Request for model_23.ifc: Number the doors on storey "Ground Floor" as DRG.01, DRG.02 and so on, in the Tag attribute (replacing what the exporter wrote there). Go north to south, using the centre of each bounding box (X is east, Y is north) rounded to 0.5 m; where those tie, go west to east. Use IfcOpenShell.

First a look at what the model holds.

```python
import ifcopenshell
import ifcopenshell.util.element
import ifcopenshell.util.placement

model = ifcopenshell.open("model_23.ifc")
print(model.schema)
storey = next(s for s in model.by_type("IfcBuildingStorey") if s.Name == "Ground Floor")
doors = [e for e in ifcopenshell.util.element.get_decomposition(storey) if e.is_a("IfcDoor")]
for e in sorted(doors, key=lambda e: e.id()):
    origin = ifcopenshell.util.placement.get_local_placement(e.ObjectPlacement)[:3, 3]
    print(e.id(), e.Tag, e.Name, origin.round(2) + 0.0, sep=" | ")
```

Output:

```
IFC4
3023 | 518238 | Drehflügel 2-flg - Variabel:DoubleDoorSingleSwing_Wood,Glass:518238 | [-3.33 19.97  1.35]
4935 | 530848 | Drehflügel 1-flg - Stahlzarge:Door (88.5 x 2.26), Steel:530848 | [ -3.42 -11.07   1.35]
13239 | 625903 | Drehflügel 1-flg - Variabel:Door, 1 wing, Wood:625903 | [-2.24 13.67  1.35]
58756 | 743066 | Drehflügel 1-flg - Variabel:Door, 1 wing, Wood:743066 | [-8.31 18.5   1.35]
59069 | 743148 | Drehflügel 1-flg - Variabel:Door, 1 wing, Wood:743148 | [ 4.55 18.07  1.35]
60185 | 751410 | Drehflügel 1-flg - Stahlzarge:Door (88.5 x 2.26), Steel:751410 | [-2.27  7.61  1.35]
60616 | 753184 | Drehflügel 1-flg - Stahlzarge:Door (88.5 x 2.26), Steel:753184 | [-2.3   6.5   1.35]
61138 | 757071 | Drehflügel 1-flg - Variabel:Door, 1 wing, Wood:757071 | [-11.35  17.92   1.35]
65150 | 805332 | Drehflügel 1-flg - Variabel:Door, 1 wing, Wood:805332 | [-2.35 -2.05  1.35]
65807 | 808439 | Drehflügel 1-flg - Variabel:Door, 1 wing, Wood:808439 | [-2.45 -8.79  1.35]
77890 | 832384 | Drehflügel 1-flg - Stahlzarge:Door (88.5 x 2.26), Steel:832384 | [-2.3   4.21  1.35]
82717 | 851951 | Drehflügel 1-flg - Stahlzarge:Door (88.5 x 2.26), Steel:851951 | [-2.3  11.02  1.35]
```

```python
import ifcopenshell
import ifcopenshell.geom
import ifcopenshell.util.element
import ifcopenshell.util.shape

model = ifcopenshell.open("model_23.ifc")
settings = ifcopenshell.geom.settings()
settings.set("use-world-coords", True)


def centre(element):
    shape = ifcopenshell.geom.create_shape(settings, element)
    return ifcopenshell.util.shape.get_bbox_centroid(shape.geometry)


storey = next(s for s in model.by_type("IfcBuildingStorey") if s.Name == "Ground Floor")
doors = [e for e in ifcopenshell.util.element.get_decomposition(storey) if e.is_a("IfcDoor")]

# Insertion points can sit at a corner or the storey origin, so sort by the geometry (in metres).
centres = {e: centre(e) for e in doors}
doors.sort(key=lambda e: (-round(centres[e][1] / 0.5), centres[e][0]))

for i, e in enumerate(doors, start=1):
    number = f"DRG.{i:02d}"
    e.Tag = number
    print(e.id(), number)

model.write("model_23_v2.ifc")
```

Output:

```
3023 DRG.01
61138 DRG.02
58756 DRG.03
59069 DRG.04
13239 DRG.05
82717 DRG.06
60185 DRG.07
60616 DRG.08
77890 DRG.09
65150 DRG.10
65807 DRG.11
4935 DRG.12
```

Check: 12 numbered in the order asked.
